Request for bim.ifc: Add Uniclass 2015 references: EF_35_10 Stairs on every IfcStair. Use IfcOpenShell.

First a look at what the model holds.

```python
import ifcopenshell

model = ifcopenshell.open("bim.ifc")
print(model.schema)
print("classifications:", [c.Name for c in model.by_type("IfcClassification")])
for ifc_class in ("IfcDoor", "IfcRoof", "IfcStair", "IfcWall", "IfcWindow"):
    print(ifc_class, len(model.by_type(ifc_class)))
```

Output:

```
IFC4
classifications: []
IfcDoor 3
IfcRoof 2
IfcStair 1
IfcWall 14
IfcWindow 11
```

```python
import ifcopenshell
import ifcopenshell.api.classification

model = ifcopenshell.open("bim.ifc")

system = ifcopenshell.api.classification.add_classification(model, classification="Uniclass 2015")

codes = {
    "IfcStair": ("EF_35_10", "Stairs"),
}
for ifc_class, (code, name) in codes.items():
    products = model.by_type(ifc_class)
    ifcopenshell.api.classification.add_reference(
        model, products=products, classification=system, identification=code, name=name
    )
    print(code, len(products))

model.write("bim_v2.ifc")
```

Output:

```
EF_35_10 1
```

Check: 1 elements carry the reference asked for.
